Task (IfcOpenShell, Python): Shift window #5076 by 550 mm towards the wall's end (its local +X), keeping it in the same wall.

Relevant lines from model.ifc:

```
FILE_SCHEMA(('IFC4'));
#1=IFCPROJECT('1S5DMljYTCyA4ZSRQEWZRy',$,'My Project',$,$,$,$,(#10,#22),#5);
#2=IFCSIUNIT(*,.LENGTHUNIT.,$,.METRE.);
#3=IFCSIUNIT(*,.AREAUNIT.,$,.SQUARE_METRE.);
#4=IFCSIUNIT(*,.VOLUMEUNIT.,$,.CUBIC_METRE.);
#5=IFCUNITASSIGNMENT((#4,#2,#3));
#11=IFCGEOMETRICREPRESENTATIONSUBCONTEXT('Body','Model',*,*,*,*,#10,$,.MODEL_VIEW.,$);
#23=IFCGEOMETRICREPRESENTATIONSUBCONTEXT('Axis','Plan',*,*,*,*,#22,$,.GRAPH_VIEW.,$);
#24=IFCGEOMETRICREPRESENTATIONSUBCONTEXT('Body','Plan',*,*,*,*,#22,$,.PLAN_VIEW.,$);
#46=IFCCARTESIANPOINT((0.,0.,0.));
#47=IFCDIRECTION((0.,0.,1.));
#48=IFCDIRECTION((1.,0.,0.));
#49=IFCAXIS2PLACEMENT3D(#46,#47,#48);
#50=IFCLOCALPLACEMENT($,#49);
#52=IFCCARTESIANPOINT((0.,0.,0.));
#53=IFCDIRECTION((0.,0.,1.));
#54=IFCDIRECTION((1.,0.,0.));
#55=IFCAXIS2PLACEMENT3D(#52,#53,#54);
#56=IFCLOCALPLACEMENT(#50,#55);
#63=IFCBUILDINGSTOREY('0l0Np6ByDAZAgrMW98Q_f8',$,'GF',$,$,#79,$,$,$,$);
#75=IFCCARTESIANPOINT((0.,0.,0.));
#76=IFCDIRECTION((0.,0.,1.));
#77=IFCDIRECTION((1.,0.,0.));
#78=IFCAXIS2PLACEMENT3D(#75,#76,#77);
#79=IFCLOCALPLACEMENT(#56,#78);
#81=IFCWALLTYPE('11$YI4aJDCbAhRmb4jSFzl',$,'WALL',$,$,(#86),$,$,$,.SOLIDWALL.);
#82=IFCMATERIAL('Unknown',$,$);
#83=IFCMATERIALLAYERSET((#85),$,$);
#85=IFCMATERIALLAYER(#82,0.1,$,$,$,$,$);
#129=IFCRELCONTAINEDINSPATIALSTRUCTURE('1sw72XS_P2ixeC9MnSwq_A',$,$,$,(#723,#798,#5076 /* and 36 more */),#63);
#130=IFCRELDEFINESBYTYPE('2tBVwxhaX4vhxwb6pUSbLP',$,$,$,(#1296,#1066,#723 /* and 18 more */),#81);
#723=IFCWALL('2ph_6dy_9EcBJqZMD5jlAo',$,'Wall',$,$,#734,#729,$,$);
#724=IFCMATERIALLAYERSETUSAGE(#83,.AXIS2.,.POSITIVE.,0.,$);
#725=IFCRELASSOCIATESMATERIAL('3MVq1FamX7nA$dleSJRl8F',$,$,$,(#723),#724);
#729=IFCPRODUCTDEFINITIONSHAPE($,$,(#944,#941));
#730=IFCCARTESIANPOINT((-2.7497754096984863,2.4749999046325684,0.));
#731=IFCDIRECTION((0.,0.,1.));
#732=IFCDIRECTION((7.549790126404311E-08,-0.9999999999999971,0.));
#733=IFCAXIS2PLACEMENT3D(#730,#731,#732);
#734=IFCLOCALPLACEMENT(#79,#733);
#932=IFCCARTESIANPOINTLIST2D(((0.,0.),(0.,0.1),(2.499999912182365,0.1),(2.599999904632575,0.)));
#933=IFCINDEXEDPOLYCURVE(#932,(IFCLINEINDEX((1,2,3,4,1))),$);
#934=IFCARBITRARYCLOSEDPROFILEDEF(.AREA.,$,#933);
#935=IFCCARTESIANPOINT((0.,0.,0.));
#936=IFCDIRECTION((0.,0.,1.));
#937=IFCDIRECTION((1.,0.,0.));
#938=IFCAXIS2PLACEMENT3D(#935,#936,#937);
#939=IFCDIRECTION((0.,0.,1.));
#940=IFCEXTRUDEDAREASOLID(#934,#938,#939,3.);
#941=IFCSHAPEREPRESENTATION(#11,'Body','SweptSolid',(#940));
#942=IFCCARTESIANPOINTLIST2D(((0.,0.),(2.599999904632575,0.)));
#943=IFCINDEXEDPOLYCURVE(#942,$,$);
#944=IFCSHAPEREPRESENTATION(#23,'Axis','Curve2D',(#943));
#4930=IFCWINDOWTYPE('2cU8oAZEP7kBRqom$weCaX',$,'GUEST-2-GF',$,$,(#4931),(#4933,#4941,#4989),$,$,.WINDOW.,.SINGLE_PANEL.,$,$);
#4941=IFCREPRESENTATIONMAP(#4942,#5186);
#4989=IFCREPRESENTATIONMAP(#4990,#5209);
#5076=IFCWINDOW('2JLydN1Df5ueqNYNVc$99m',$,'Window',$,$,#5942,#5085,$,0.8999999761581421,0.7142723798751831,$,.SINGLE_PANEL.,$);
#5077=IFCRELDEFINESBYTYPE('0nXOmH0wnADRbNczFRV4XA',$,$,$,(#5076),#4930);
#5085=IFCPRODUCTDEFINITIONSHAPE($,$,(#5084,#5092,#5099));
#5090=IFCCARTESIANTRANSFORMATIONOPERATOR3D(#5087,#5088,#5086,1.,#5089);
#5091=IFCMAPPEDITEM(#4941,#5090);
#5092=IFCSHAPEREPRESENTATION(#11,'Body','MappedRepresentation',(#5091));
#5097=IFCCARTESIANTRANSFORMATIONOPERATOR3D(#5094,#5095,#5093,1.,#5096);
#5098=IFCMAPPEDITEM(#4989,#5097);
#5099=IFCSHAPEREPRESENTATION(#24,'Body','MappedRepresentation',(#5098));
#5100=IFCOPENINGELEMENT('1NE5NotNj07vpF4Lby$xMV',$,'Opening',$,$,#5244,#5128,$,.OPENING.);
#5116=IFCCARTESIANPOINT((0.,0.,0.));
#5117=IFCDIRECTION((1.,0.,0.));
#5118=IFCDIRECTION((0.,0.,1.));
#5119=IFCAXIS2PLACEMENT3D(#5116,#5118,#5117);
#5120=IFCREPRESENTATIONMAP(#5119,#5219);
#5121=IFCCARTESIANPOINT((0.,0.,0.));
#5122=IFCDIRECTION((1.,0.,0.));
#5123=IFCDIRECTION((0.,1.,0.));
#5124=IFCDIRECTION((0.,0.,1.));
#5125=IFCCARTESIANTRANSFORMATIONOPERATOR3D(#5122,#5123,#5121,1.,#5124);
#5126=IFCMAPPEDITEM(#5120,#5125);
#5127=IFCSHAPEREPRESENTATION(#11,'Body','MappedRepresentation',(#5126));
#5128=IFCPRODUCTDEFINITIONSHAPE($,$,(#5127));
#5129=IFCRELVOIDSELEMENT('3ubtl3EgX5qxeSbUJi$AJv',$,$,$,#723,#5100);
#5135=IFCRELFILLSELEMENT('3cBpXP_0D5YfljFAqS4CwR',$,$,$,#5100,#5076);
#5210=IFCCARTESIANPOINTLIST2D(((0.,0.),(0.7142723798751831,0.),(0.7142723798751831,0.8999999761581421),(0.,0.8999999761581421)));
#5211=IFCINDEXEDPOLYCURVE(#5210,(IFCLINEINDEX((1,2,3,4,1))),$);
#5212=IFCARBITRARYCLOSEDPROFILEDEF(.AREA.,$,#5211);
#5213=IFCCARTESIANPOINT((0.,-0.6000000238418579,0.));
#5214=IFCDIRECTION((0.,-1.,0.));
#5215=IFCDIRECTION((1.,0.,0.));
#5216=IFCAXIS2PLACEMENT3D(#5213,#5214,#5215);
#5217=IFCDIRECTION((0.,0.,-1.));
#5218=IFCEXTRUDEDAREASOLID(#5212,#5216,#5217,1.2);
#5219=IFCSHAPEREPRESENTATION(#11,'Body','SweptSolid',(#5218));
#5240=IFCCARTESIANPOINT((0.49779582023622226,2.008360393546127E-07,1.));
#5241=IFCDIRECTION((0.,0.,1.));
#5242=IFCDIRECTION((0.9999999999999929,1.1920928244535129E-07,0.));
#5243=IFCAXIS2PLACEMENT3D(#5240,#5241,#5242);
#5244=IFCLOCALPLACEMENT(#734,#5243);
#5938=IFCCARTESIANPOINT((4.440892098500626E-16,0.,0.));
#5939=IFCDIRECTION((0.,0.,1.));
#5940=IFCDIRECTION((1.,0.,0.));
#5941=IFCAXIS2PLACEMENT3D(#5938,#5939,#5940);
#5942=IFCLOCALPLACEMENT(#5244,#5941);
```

```python
import ifcopenshell
import ifcopenshell.api.geometry
import ifcopenshell.util.placement
import ifcopenshell.util.unit

model = ifcopenshell.open("model.ifc")
unit_scale = ifcopenshell.util.unit.calculate_unit_scale(model)

window = model.by_guid("2JLydN1Df5ueqNYNVc$99m")
opening = window.FillsVoids[0].RelatingOpeningElement
wall = opening.VoidsElements[0].RelatingBuildingElement

wall_matrix = ifcopenshell.util.placement.get_local_placement(wall.ObjectPlacement)
shift = wall_matrix[:3, 0] * 0.55 / unit_scale
before = ifcopenshell.util.placement.get_local_placement(window.ObjectPlacement)[:3, 3].copy()

# The window is placed relative to its opening, so it follows when the opening moves.
matrix = ifcopenshell.util.placement.get_local_placement(opening.ObjectPlacement)
matrix[:3, 3] += shift
ifcopenshell.api.geometry.edit_object_placement(
    model, product=opening, matrix=matrix, is_si=False, should_transform_children=True
)

after = ifcopenshell.util.placement.get_local_placement(window.ObjectPlacement)[:3, 3]
print("window moved by", (after - before).round(3) + 0.0)

model.write("model_updated.ifc")
```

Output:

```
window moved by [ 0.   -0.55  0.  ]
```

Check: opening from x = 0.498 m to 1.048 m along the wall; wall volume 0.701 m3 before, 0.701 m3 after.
